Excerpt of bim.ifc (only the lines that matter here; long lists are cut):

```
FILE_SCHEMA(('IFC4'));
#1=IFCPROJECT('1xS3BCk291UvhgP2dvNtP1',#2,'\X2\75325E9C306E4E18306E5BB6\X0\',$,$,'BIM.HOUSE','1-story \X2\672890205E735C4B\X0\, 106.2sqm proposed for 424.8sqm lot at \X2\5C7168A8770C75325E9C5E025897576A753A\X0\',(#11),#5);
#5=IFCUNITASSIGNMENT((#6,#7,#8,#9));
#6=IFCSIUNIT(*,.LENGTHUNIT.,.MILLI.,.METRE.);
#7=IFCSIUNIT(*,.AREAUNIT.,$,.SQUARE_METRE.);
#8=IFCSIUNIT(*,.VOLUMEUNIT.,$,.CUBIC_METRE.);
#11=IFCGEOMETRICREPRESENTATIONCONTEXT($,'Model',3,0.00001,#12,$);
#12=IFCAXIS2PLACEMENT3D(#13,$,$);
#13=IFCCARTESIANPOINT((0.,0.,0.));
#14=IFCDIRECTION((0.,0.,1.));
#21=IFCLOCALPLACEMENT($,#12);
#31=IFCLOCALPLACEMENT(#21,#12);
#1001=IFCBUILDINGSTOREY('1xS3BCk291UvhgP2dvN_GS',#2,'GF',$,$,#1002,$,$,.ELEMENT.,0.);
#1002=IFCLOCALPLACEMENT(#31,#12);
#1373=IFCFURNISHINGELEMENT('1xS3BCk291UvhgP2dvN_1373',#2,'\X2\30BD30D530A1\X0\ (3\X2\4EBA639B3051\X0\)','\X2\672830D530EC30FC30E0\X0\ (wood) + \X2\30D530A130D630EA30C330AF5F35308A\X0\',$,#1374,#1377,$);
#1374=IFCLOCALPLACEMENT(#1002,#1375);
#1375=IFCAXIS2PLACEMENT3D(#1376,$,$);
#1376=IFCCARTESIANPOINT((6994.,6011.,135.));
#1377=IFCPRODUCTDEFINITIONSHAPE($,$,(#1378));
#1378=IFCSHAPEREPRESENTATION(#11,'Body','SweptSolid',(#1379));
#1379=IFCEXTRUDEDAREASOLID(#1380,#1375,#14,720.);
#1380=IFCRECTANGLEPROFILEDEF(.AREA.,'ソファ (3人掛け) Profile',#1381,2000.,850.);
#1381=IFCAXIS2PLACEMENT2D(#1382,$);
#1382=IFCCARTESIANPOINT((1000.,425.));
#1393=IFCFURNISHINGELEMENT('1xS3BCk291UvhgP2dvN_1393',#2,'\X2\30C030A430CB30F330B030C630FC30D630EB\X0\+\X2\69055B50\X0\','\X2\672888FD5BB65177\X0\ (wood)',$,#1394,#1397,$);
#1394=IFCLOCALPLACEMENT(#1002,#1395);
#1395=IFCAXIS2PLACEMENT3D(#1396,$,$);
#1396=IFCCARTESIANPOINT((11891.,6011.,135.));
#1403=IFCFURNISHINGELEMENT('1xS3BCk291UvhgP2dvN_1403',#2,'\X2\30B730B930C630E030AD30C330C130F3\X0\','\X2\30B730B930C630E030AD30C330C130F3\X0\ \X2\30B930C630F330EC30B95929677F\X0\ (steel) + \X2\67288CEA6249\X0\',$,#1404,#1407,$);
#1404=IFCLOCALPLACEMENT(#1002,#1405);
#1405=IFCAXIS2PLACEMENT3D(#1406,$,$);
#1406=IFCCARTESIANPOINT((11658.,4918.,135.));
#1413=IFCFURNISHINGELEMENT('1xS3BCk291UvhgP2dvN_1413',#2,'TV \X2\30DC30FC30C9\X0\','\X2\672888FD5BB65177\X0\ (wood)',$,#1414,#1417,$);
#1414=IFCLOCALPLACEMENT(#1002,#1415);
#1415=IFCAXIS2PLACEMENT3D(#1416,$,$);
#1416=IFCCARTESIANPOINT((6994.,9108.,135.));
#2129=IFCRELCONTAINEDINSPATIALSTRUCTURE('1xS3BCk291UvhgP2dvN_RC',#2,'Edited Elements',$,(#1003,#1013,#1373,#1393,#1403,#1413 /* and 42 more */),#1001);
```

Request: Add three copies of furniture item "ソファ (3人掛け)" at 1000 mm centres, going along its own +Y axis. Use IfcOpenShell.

```python
import ifcopenshell
import ifcopenshell.api.geometry
import ifcopenshell.api.root
import ifcopenshell.util.element
import ifcopenshell.util.placement
import ifcopenshell.util.unit

model = ifcopenshell.open("bim.ifc")
unit_scale = ifcopenshell.util.unit.calculate_unit_scale(model)


def reuse_history(source, copy):
    """copy_class also copies each property set's owner history, people and application; keep the originals."""
    for rel in copy.IsDefinedBy:
        if rel.is_a("IfcRelDefinesByProperties") and (history := rel.RelatingPropertyDefinition.OwnerHistory):
            rel.RelatingPropertyDefinition.OwnerHistory = source.OwnerHistory
            ifcopenshell.util.element.remove_deep2(model, history)


source = model.by_guid("1xS3BCk291UvhgP2dvN_1373")
base = ifcopenshell.util.placement.get_local_placement(source.ObjectPlacement)
step = base[:3, 1] * 1 / unit_scale

for i in range(1, 4):
    copy = ifcopenshell.api.root.copy_class(model, product=source)
    copy.Representation = ifcopenshell.util.element.copy_deep(
        model, source.Representation, exclude=["IfcGeometricRepresentationContext", "IfcRepresentationMap"]
    )
    reuse_history(source, copy)
    matrix = base.copy()
    matrix[:3, 3] += i * step
    print("added at", matrix[:3, 3].round(3) + 0.0)
    ifcopenshell.api.geometry.edit_object_placement(model, product=copy, matrix=matrix, is_si=False)

model.write("bim_updated.ifc")
```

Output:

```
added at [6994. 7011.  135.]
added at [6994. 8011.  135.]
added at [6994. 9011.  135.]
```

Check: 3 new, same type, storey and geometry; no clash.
